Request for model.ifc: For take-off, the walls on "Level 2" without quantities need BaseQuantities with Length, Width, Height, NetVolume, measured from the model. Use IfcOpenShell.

First a look at what the model holds.

```python
import ifcopenshell
import ifcopenshell.util.element
import ifcopenshell.util.unit

model = ifcopenshell.open("model.ifc")
print(model.schema)
for unit_type in ("LENGTHUNIT", "AREAUNIT", "VOLUMEUNIT"):
    print(unit_type, ifcopenshell.util.unit.calculate_unit_scale(model, unit_type))
storey = next(s for s in model.by_type("IfcBuildingStorey") if s.Name == "Level 2")
walls = [e for e in ifcopenshell.util.element.get_decomposition(storey) if e.is_a("IfcWall")]
for e in sorted(walls, key=lambda e: e.id()):
    print(e.id(), e.is_a(), e.Name, list(ifcopenshell.util.element.get_psets(e, qtos_only=True)), sep=" | ")
```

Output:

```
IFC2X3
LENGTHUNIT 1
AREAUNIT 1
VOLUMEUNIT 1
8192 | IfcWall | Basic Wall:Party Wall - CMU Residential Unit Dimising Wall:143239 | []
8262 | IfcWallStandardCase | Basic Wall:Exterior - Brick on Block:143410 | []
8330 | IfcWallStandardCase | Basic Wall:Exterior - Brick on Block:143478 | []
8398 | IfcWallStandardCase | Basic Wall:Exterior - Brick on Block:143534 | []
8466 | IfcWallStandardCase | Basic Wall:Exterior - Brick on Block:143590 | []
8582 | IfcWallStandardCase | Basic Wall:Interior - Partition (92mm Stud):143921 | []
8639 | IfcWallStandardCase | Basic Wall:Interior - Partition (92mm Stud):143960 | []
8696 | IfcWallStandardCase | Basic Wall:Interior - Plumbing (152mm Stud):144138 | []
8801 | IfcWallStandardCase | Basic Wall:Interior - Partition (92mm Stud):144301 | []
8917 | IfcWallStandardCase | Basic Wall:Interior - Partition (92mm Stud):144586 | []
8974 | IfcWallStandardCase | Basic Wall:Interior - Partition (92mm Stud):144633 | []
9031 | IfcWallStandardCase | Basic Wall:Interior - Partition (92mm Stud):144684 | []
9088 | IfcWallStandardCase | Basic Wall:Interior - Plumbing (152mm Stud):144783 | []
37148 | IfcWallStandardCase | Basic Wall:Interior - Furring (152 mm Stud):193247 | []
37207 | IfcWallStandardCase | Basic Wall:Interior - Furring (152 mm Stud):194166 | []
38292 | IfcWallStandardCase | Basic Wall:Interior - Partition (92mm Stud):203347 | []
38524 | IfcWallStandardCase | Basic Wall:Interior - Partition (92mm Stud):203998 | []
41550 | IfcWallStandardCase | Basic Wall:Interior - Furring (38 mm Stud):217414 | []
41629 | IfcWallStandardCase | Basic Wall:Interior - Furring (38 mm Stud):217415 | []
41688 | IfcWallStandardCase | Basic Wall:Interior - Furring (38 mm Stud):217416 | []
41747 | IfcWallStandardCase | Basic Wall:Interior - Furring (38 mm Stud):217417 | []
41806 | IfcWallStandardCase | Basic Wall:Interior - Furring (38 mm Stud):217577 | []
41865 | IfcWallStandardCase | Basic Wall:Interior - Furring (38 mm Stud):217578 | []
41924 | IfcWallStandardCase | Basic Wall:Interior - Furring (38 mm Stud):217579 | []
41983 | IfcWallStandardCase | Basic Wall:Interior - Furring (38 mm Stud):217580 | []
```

```python
import ifcopenshell
import ifcopenshell.api.pset
import ifcopenshell.geom
import ifcopenshell.util.element
import ifcopenshell.util.shape
import ifcopenshell.util.unit

model = ifcopenshell.open("model.ifc")
unit_scale = ifcopenshell.util.unit.calculate_unit_scale(model)
volume_scale = ifcopenshell.util.unit.calculate_unit_scale(model, "VOLUMEUNIT")
settings = ifcopenshell.geom.settings()

storey = next(s for s in model.by_type("IfcBuildingStorey") if s.Name == "Level 2")
walls = [e for e in ifcopenshell.util.element.get_decomposition(storey) if e.is_a("IfcWall")]

for e in sorted(walls, key=lambda e: e.id()):
    if ifcopenshell.util.element.get_psets(e, qtos_only=True, should_inherit=False):
        continue
    # Geometry comes back in metres, in the element's own axes.
    shape = ifcopenshell.geom.create_shape(settings, e)
    values = {
        "Length": ifcopenshell.util.shape.get_x(shape.geometry) / unit_scale,
        "Width": ifcopenshell.util.shape.get_y(shape.geometry) / unit_scale,
        "Height": ifcopenshell.util.shape.get_z(shape.geometry) / unit_scale,
        "NetVolume": ifcopenshell.util.shape.get_volume(shape.geometry) / volume_scale,
    }
    qto = ifcopenshell.api.pset.add_qto(model, product=e, name="BaseQuantities")
    ifcopenshell.api.pset.edit_qto(model, qto=qto, properties=values)
    print(e.id(), {k: round(v, 3) for k, v in values.items()})

model.write("model_rev.ifc")
```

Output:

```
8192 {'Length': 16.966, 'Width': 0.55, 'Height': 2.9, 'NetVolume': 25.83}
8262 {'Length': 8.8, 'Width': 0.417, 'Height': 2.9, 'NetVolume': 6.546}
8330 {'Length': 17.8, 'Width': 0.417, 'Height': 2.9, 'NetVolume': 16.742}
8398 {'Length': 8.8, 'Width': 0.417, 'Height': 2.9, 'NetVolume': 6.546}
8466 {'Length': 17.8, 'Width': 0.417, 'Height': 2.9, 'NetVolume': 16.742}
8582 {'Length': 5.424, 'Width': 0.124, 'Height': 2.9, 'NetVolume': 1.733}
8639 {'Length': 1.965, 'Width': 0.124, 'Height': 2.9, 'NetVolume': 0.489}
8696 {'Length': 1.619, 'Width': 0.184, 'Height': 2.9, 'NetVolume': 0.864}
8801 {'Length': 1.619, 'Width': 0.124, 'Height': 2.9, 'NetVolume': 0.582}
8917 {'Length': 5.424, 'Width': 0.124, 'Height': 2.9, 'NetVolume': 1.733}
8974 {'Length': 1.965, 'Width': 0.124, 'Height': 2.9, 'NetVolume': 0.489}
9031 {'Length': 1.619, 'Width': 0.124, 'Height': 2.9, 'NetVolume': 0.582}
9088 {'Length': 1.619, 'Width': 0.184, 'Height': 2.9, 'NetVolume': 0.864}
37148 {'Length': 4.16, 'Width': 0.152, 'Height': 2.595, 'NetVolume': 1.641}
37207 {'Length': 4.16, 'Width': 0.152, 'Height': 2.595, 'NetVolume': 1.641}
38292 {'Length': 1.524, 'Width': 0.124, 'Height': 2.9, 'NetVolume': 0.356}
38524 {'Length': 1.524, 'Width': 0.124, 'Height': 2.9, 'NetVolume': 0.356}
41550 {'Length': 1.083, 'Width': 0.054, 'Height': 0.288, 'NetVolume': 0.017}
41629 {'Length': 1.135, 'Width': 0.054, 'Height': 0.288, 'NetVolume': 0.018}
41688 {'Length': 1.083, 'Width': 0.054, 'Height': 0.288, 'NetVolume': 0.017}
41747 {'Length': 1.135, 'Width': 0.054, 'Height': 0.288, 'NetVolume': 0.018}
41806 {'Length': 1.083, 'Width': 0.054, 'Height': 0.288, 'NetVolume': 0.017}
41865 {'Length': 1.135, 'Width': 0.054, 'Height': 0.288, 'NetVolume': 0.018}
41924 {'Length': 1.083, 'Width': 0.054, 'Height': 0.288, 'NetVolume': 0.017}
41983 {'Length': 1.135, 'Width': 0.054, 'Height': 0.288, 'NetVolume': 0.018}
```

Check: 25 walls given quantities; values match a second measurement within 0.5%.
